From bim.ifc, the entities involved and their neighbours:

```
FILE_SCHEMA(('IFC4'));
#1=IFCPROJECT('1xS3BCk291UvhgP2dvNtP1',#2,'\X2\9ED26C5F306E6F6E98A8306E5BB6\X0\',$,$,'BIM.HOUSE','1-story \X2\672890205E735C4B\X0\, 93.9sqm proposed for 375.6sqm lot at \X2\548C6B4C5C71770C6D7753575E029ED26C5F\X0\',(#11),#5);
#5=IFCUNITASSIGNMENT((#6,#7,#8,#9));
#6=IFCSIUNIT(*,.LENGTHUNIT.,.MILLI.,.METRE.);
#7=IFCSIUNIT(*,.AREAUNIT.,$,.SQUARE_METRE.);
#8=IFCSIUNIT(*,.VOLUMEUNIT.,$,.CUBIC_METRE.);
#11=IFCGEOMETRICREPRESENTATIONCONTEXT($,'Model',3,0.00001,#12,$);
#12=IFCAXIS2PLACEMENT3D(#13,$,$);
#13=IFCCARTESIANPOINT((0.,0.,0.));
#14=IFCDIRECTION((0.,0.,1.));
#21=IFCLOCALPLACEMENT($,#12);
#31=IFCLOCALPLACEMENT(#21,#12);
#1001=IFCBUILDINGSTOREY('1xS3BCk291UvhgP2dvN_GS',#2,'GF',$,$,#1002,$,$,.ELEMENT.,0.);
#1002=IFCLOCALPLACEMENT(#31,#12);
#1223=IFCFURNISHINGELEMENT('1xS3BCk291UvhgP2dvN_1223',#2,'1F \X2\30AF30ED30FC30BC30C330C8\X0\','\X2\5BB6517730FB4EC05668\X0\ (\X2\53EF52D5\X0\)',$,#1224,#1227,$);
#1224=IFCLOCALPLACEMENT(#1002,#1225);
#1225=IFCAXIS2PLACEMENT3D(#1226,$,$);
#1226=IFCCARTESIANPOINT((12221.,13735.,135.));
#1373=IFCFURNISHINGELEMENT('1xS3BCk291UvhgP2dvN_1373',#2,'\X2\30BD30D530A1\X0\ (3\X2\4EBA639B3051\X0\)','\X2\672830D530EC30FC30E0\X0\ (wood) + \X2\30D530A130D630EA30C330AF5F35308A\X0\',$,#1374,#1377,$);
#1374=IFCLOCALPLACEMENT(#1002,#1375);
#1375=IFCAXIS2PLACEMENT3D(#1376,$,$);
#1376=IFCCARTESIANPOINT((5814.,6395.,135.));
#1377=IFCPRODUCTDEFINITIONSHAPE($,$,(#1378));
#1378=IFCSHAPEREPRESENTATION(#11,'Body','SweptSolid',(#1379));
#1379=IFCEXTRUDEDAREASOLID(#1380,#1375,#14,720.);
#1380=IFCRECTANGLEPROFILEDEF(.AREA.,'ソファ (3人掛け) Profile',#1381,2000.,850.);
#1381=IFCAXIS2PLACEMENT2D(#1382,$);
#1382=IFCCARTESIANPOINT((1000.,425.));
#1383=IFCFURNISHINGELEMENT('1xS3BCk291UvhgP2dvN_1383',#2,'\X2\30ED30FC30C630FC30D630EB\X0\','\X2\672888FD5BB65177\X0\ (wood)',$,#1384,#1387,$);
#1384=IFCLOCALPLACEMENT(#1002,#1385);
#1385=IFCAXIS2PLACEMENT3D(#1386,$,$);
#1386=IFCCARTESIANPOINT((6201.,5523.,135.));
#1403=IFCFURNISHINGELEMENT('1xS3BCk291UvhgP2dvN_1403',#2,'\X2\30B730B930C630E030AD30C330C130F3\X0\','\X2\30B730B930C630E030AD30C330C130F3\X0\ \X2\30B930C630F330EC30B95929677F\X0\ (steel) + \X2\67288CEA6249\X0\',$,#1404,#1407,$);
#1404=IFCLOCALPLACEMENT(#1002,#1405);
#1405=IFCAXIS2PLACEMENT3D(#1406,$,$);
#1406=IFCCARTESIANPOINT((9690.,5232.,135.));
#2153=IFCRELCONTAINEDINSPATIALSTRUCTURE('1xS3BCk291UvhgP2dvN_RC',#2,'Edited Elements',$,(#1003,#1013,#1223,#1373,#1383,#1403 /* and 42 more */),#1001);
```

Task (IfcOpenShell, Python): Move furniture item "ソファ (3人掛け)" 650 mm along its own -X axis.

```python
import ifcopenshell
import ifcopenshell.api.geometry
import ifcopenshell.util.placement
import ifcopenshell.util.unit

model = ifcopenshell.open("bim.ifc")
unit_scale = ifcopenshell.util.unit.calculate_unit_scale(model)

item = model.by_guid("1xS3BCk291UvhgP2dvN_1373")
matrix = ifcopenshell.util.placement.get_local_placement(item.ObjectPlacement)
matrix[:3, 3] -= matrix[:3, 0] * 0.65 / unit_scale
ifcopenshell.api.geometry.edit_object_placement(model, product=item, matrix=matrix, is_si=False)

print(ifcopenshell.util.placement.get_local_placement(item.ObjectPlacement).round(3) + 0.0)

model.write("bim_v2.ifc")
```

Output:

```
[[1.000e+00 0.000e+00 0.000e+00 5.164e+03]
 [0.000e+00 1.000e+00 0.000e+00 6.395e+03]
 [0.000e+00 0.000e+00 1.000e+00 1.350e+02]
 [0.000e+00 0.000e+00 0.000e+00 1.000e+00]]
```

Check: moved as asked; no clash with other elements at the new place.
